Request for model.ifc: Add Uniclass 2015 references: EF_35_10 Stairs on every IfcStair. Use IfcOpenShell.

First a look at what the model holds.

```python
import ifcopenshell

model = ifcopenshell.open("model.ifc")
print(model.schema)
print("classifications:", [c.Name for c in model.by_type("IfcClassification")])
for ifc_class in ("IfcDoor", "IfcRoof", "IfcStair", "IfcWall", "IfcWindow"):
    print(ifc_class, len(model.by_type(ifc_class)))
```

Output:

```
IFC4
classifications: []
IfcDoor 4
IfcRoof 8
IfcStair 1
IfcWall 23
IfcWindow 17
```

```python
import ifcopenshell
import ifcopenshell.api.classification

model = ifcopenshell.open("model.ifc")

system = ifcopenshell.api.classification.add_classification(model, classification="Uniclass 2015")

codes = {
    "IfcStair": ("EF_35_10", "Stairs"),
}
for ifc_class, (code, name) in codes.items():
    products = model.by_type(ifc_class)
    ifcopenshell.api.classification.add_reference(
        model, products=products, classification=system, identification=code, name=name
    )
    print(code, len(products))

model.write("model_v2.ifc")
```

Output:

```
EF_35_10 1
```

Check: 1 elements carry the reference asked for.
